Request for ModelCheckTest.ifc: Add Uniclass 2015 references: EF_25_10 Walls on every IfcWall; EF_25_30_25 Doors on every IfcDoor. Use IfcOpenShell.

First a look at what the model holds.

```python
import ifcopenshell

model = ifcopenshell.open("ModelCheckTest.ifc")
print(model.schema)
print("classifications:", [c.Name for c in model.by_type("IfcClassification")])
for ifc_class in ("IfcDoor", "IfcRoof", "IfcStair", "IfcWall", "IfcWindow"):
    print(ifc_class, len(model.by_type(ifc_class)))
```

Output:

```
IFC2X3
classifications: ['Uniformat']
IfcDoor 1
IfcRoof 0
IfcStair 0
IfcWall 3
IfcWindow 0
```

```python
import ifcopenshell
import ifcopenshell.api.classification

model = ifcopenshell.open("ModelCheckTest.ifc")

# IFC2X3 requires Source and Edition and has no link from the project to the system.
system = model.create_entity("IfcClassification", Source="NBS", Edition="2015", Name="Uniclass 2015")

codes = {
    "IfcWall": ("EF_25_10", "Walls"),
    "IfcDoor": ("EF_25_30_25", "Doors"),
}
for ifc_class, (code, name) in codes.items():
    products = model.by_type(ifc_class)
    ifcopenshell.api.classification.add_reference(
        model, products=products, classification=system, identification=code, name=name
    )
    print(code, len(products))

model.write("ModelCheckTest-out.ifc")
```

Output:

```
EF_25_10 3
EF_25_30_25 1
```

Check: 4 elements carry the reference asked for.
